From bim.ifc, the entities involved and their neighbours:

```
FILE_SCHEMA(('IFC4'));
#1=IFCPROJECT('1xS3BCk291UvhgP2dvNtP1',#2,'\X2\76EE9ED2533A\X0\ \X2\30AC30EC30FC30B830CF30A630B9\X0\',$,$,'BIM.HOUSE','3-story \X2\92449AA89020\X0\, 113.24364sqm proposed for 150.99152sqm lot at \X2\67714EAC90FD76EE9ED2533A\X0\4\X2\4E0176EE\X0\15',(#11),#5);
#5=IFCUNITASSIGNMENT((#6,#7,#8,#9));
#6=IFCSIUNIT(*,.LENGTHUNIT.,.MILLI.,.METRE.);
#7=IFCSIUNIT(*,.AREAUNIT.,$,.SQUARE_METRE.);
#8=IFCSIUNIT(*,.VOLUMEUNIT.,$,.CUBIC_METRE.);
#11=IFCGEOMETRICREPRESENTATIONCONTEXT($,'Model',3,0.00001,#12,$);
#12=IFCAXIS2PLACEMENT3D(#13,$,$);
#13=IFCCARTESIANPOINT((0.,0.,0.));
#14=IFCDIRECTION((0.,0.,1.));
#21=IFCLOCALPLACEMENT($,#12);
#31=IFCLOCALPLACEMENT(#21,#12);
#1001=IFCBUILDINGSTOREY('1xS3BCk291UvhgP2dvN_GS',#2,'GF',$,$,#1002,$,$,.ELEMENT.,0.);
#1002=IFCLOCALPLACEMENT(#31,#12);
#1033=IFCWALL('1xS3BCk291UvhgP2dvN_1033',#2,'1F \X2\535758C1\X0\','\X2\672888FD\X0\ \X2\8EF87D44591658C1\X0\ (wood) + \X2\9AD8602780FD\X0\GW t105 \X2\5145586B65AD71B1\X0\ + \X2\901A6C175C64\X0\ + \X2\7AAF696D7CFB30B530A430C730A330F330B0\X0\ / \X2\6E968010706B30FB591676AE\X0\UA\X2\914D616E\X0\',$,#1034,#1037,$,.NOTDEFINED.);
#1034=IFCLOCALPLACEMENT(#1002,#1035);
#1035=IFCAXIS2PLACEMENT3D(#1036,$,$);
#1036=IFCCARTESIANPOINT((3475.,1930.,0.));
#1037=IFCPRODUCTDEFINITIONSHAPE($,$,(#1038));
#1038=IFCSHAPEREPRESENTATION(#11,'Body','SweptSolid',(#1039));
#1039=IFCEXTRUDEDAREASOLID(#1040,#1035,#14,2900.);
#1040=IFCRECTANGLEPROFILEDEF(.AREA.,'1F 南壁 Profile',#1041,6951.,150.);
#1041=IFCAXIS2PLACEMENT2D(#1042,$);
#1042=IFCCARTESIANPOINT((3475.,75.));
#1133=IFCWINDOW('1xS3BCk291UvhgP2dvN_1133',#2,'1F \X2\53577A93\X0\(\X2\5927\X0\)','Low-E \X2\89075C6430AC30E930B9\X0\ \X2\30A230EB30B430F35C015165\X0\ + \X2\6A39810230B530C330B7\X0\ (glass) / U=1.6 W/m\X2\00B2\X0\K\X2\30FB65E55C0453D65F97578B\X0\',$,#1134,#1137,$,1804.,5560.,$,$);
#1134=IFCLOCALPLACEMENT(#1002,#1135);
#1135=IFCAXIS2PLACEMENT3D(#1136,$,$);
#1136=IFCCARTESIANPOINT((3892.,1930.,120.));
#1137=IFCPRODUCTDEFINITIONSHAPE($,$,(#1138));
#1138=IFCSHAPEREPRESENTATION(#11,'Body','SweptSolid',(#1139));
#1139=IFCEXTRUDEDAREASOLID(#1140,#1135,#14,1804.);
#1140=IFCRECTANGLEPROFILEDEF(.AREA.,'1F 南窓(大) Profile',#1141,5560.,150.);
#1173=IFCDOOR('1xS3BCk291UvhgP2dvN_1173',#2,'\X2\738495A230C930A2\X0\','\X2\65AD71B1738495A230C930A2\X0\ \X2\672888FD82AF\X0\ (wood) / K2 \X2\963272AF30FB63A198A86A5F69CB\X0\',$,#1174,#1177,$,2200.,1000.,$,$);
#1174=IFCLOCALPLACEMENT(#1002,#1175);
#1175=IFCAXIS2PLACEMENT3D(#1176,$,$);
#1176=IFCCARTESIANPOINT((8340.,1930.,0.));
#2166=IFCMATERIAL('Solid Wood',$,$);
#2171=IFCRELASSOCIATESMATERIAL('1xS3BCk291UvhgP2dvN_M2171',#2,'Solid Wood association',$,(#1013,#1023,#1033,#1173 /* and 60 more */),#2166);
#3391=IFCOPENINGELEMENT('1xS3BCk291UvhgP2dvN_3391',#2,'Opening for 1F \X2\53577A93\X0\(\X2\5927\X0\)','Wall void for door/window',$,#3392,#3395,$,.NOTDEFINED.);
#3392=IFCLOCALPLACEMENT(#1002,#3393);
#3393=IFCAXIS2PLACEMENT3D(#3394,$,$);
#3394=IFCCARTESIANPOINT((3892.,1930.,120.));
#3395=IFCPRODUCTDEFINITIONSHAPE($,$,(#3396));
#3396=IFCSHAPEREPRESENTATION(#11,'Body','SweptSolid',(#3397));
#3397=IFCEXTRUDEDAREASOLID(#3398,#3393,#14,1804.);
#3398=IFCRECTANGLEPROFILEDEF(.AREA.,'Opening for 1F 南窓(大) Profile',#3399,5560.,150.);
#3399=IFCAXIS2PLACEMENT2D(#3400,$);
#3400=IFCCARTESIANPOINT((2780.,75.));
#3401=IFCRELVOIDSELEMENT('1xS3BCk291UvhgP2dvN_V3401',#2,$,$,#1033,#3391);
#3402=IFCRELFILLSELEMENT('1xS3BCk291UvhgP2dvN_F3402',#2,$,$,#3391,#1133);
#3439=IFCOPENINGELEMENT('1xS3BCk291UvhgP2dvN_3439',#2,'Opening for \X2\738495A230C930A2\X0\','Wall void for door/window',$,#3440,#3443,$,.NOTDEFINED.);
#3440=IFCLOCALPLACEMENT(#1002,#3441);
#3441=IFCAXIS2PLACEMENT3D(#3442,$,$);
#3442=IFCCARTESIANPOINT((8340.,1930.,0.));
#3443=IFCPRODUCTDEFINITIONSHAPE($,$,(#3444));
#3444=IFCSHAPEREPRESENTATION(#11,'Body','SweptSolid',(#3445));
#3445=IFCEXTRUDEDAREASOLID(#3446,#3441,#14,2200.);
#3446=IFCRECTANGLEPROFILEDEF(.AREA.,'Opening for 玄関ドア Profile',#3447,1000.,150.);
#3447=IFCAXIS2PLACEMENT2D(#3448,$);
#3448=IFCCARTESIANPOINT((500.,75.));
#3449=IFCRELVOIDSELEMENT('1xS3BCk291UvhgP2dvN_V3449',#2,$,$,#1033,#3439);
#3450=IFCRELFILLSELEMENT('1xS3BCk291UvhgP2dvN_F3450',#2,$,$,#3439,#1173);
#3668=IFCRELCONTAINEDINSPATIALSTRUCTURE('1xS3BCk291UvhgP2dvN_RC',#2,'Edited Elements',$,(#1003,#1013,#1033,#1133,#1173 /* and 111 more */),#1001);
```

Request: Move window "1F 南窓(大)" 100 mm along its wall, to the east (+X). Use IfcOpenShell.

```python
import ifcopenshell
import ifcopenshell.api.geometry
import ifcopenshell.util.placement

model = ifcopenshell.open("bim.ifc")

window = model.by_guid("1xS3BCk291UvhgP2dvN_1133")
opening = window.FillsVoids[0].RelatingOpeningElement
wall = opening.VoidsElements[0].RelatingBuildingElement

wall_matrix = ifcopenshell.util.placement.get_local_placement(wall.ObjectPlacement)
shift = wall_matrix[:3, 0] * 100.0
before = ifcopenshell.util.placement.get_local_placement(window.ObjectPlacement)[:3, 3].copy()

# The window is not placed relative to its opening, so move both.
for product in (opening, window):
    matrix = ifcopenshell.util.placement.get_local_placement(product.ObjectPlacement)
    matrix[:3, 3] += shift
    ifcopenshell.api.geometry.edit_object_placement(model, product=product, matrix=matrix, is_si=False)

after = ifcopenshell.util.placement.get_local_placement(window.ObjectPlacement)[:3, 3]
print("window moved by", (after - before).round(3) + 0.0)

model.write("bim_rev.ifc")
```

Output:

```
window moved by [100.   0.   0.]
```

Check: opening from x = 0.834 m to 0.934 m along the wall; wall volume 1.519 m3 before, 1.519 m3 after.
